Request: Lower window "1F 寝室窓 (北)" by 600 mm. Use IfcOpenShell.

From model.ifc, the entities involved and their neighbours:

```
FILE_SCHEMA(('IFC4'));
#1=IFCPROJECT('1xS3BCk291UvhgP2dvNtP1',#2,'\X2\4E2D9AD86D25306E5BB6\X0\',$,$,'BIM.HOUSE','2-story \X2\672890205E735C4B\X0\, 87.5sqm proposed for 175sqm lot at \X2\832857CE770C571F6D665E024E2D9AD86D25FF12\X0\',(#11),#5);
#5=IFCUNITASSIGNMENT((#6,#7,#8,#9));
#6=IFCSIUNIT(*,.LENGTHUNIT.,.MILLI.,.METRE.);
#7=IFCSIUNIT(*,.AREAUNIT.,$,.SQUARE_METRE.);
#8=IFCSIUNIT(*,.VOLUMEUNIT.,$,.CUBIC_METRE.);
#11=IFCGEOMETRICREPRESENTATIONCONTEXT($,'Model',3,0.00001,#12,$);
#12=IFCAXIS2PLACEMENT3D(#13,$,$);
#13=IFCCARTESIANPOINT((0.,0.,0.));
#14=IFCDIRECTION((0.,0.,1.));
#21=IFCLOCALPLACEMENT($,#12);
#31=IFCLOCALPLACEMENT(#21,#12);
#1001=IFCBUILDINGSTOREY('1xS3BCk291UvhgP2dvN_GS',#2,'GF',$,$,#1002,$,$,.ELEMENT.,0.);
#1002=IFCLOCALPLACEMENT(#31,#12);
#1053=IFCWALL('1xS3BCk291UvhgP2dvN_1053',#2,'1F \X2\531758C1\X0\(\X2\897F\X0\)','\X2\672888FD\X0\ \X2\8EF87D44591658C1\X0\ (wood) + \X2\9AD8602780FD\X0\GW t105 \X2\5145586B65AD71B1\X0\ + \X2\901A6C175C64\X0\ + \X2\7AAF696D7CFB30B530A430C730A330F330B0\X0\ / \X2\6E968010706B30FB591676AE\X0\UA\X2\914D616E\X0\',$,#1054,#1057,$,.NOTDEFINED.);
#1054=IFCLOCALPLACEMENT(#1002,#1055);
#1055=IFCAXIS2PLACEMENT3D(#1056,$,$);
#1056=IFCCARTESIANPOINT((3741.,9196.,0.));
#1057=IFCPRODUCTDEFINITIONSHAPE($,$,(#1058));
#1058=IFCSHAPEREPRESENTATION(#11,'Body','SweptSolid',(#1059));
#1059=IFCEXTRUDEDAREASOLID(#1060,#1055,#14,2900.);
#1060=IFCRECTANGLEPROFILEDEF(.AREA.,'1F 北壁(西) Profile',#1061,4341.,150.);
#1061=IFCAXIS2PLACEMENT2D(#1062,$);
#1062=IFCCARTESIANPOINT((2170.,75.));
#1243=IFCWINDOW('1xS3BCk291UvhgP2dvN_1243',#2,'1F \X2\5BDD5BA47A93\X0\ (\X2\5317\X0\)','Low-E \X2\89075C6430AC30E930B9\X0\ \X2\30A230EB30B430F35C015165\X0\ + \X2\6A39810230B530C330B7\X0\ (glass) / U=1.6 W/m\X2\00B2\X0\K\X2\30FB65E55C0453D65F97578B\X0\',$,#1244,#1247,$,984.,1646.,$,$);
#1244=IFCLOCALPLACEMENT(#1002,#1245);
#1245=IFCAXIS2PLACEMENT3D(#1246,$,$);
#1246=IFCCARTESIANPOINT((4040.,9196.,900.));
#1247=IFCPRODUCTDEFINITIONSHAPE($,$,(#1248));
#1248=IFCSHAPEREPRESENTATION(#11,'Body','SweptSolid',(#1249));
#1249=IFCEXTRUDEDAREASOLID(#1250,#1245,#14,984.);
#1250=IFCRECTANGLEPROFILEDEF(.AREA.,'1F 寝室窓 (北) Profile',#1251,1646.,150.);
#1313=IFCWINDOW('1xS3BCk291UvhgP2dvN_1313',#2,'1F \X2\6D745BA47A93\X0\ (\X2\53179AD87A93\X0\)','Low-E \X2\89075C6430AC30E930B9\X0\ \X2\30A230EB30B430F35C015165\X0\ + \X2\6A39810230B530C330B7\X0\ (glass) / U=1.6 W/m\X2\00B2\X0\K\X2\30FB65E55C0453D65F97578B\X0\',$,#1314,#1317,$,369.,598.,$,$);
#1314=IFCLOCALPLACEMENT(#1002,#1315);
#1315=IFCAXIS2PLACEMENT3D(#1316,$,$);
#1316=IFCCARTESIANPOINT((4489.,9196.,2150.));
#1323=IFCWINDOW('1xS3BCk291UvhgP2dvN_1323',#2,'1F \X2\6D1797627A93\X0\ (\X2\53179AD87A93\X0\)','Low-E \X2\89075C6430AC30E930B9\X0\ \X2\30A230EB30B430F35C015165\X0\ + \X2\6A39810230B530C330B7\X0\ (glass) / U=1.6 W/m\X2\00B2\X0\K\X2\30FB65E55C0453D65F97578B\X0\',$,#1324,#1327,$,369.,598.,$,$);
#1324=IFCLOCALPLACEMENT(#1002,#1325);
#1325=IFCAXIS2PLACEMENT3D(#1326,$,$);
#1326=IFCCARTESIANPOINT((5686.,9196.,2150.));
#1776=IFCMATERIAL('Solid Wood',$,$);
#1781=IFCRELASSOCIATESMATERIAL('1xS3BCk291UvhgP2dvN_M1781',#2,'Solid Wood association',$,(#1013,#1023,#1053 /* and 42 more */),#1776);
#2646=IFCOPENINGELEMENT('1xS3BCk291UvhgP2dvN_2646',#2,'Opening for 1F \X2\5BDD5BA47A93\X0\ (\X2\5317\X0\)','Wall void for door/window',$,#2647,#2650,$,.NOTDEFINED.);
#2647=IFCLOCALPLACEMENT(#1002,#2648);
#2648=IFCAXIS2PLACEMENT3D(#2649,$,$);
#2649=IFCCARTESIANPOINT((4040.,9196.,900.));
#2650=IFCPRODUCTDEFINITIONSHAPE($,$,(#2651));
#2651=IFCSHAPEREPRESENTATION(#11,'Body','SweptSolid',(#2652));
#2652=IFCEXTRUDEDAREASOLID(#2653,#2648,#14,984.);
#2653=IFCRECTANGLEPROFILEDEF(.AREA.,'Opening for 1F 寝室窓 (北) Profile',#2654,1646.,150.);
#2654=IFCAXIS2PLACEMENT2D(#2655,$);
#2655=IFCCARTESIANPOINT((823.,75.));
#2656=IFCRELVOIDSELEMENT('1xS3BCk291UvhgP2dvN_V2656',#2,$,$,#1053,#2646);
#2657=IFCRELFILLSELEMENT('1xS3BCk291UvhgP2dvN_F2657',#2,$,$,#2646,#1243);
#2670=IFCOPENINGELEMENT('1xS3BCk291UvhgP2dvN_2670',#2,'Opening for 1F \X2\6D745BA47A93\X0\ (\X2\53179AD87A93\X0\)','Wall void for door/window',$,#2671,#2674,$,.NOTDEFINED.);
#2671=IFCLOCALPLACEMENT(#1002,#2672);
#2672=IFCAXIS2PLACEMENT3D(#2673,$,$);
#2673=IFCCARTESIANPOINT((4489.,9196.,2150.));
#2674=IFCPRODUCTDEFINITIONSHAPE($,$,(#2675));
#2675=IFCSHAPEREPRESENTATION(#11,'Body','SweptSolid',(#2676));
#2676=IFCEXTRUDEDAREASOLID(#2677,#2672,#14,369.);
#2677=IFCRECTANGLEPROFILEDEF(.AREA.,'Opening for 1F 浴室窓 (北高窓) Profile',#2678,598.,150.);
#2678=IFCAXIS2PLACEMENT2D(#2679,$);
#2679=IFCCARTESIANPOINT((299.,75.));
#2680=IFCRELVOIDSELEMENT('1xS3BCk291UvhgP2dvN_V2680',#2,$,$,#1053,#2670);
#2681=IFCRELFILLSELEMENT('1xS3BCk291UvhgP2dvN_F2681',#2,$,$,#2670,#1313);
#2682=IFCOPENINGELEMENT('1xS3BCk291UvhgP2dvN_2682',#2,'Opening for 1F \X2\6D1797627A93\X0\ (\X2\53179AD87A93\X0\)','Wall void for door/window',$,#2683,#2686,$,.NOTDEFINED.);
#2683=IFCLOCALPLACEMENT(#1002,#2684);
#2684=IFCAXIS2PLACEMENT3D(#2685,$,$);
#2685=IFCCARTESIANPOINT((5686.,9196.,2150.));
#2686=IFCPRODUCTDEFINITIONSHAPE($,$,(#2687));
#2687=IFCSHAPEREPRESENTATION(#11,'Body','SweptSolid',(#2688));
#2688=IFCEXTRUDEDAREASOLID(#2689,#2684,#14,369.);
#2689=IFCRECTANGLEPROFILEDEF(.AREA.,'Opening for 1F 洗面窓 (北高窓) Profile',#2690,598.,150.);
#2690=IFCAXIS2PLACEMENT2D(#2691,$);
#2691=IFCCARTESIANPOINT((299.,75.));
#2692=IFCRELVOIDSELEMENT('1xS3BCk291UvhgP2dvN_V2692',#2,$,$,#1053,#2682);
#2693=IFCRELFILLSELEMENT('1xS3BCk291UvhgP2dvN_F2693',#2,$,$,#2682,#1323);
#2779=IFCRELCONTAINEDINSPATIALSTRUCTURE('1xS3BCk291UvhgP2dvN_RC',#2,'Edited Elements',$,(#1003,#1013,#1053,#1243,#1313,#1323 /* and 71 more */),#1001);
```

```python
import numpy as np
import ifcopenshell
import ifcopenshell.api.geometry
import ifcopenshell.util.placement
import ifcopenshell.util.unit

model = ifcopenshell.open("model.ifc")
unit_scale = ifcopenshell.util.unit.calculate_unit_scale(model)

window = model.by_guid("1xS3BCk291UvhgP2dvN_1243")
opening = window.FillsVoids[0].RelatingOpeningElement
dz = -0.6 / unit_scale

shift = np.array([0.0, 0.0, dz])
# The window is not placed relative to its opening, so move both.
for product in (opening, window):
    matrix = ifcopenshell.util.placement.get_local_placement(product.ObjectPlacement)
    matrix[:3, 3] += shift
    ifcopenshell.api.geometry.edit_object_placement(model, product=product, matrix=matrix, is_si=False)

print(f"moved by {dz * unit_scale:+.3f} m")

model.write("model_updated.ifc")
```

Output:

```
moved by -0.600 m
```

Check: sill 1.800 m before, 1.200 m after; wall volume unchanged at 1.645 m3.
